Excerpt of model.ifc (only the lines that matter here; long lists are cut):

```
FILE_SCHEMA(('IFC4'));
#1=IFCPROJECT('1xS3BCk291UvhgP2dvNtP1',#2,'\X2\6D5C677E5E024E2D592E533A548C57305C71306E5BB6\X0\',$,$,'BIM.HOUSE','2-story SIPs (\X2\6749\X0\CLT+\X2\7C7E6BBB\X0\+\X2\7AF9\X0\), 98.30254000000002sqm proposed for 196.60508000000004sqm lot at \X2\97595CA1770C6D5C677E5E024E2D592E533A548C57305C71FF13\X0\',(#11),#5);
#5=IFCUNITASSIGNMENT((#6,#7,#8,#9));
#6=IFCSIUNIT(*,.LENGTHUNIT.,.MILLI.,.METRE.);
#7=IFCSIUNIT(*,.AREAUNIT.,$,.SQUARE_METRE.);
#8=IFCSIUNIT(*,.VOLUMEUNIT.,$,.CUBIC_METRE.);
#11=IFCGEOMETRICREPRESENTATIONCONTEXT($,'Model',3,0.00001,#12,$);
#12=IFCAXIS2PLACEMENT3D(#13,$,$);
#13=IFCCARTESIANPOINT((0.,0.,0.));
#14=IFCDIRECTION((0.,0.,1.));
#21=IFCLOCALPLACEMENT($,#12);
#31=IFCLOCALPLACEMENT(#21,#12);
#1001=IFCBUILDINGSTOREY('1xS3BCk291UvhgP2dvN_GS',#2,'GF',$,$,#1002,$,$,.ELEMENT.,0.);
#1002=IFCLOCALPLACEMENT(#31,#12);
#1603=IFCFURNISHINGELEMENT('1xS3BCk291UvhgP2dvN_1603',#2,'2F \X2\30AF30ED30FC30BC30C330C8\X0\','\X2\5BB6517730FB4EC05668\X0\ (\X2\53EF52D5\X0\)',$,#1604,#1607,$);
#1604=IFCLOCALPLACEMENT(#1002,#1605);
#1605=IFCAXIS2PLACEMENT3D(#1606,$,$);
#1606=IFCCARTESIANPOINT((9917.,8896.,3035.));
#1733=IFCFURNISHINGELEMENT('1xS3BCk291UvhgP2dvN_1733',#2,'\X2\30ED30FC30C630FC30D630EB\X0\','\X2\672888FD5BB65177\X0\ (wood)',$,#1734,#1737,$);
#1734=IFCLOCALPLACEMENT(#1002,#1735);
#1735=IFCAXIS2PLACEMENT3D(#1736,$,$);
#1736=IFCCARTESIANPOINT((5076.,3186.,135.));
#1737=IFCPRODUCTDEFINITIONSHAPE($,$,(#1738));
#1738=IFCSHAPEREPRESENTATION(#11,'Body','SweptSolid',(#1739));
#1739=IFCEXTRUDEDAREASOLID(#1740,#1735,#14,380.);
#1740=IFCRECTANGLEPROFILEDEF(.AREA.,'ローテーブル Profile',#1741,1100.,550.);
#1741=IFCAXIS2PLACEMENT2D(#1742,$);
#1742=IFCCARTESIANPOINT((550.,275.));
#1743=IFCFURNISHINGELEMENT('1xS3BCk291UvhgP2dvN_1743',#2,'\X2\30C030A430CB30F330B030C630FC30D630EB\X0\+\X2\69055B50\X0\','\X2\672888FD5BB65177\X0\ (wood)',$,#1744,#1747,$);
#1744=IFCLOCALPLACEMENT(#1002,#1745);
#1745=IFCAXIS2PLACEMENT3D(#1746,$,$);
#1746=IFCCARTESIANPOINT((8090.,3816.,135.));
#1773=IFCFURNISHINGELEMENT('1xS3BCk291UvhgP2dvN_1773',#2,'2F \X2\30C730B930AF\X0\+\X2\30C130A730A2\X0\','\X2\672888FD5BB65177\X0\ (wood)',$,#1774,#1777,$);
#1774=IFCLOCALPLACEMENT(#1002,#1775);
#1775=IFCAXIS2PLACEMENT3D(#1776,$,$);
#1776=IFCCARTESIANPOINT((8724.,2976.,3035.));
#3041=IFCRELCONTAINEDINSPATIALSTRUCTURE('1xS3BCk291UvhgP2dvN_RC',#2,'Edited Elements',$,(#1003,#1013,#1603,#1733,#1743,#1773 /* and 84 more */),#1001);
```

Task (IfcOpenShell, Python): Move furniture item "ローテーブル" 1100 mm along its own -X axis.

```python
import ifcopenshell
import ifcopenshell.api.geometry
import ifcopenshell.util.placement
import ifcopenshell.util.unit

model = ifcopenshell.open("model.ifc")
unit_scale = ifcopenshell.util.unit.calculate_unit_scale(model)

item = model.by_guid("1xS3BCk291UvhgP2dvN_1733")
matrix = ifcopenshell.util.placement.get_local_placement(item.ObjectPlacement)
matrix[:3, 3] -= matrix[:3, 0] * 1.1 / unit_scale
ifcopenshell.api.geometry.edit_object_placement(model, product=item, matrix=matrix, is_si=False)

print(ifcopenshell.util.placement.get_local_placement(item.ObjectPlacement).round(3) + 0.0)

model.write("model_v2.ifc")
```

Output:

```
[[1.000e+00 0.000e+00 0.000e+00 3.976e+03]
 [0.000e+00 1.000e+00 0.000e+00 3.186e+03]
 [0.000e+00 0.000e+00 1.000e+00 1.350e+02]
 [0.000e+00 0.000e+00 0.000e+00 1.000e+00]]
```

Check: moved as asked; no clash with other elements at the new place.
